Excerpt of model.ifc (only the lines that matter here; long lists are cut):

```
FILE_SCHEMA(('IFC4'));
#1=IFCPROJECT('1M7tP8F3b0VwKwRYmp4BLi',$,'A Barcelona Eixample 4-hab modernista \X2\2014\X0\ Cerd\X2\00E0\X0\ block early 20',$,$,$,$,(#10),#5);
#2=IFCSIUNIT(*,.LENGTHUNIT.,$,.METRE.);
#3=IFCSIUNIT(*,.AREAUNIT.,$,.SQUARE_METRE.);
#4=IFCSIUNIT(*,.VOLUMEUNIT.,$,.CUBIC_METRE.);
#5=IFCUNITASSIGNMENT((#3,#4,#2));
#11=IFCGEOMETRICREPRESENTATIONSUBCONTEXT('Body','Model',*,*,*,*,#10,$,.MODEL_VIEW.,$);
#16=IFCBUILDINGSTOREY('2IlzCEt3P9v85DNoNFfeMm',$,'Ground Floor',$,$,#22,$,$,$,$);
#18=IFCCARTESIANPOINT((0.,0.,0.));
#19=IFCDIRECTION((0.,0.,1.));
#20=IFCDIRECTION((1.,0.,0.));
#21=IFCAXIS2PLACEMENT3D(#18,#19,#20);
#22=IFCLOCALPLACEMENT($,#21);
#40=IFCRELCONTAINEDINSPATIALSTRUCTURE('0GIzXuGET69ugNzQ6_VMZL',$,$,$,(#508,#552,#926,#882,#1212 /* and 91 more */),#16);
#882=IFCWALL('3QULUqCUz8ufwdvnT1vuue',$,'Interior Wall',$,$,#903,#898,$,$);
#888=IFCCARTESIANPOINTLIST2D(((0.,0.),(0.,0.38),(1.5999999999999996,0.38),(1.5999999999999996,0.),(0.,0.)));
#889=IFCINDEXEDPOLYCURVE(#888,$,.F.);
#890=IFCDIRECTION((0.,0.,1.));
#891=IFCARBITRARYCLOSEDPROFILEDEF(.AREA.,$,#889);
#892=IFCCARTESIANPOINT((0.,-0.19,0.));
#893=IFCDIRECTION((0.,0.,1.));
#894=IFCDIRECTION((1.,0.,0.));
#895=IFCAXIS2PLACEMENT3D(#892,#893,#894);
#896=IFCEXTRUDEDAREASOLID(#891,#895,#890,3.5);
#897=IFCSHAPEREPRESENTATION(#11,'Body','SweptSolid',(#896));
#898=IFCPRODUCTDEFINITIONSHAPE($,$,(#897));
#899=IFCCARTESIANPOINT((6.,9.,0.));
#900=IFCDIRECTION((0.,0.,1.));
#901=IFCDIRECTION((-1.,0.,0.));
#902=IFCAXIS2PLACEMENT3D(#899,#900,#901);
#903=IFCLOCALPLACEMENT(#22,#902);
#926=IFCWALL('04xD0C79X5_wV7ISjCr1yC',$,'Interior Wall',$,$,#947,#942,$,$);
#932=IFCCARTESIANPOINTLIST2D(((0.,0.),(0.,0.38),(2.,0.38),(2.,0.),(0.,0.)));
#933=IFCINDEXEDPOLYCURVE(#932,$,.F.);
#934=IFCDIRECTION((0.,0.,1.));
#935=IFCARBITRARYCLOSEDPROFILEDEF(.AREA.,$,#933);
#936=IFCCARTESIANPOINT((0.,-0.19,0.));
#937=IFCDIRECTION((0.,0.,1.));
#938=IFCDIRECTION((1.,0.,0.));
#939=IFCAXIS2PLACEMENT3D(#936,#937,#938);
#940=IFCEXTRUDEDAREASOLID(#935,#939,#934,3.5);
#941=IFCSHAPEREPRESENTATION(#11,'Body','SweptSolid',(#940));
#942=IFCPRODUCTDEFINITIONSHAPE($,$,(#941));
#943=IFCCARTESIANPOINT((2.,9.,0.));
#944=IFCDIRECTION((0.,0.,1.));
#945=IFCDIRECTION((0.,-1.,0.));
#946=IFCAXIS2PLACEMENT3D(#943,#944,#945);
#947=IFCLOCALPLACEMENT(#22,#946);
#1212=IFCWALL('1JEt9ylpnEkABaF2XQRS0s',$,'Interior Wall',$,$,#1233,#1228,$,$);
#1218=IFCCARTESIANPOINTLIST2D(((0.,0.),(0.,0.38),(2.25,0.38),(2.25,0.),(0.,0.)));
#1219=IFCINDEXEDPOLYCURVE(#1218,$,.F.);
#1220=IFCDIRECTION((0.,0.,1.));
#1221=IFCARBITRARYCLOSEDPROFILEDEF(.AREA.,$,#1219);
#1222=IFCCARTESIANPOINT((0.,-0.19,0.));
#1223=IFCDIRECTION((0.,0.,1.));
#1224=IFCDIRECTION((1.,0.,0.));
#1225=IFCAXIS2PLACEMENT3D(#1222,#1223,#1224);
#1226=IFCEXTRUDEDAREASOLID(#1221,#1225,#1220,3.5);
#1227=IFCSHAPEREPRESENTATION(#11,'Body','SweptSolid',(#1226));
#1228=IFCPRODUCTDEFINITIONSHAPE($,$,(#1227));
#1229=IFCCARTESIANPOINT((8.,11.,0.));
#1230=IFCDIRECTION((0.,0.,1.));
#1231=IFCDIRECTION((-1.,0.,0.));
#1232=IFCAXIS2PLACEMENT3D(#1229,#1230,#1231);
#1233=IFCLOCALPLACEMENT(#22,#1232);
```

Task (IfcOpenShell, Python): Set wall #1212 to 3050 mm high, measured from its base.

```python
import ifcopenshell
import ifcopenshell.geom
import ifcopenshell.util.representation
import ifcopenshell.util.shape
import ifcopenshell.util.unit

model = ifcopenshell.open("model.ifc")
unit_scale = ifcopenshell.util.unit.calculate_unit_scale(model)
settings = ifcopenshell.geom.settings()


def volume(element):
    """Net volume in cubic metres, openings subtracted."""
    shape = ifcopenshell.geom.create_shape(settings, element)
    return ifcopenshell.util.shape.get_volume(shape.geometry)


wall = model.by_id(1212)
before = volume(wall)

body = ifcopenshell.util.representation.get_representation(wall, "Model", "Body")
solid = body.Items[0]
old_height = solid.Depth
solid.Depth = 3.05 / unit_scale
after = volume(wall)

print(f"height {old_height:g} -> {solid.Depth:g}, volume {before:.3f} -> {after:.3f} m3")

model.write("model-out.ifc")
```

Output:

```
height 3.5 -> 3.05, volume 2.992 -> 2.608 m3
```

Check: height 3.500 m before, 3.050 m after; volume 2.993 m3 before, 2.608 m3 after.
